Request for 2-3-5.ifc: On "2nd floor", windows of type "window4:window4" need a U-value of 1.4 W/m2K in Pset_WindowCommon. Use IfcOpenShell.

First a look at what the model holds.

```python
import ifcopenshell
import ifcopenshell.util.element

model = ifcopenshell.open("2-3-5.ifc")
print(model.schema)
storey = next(s for s in model.by_type("IfcBuildingStorey") if s.Name == "2nd floor")
windows = [e for e in ifcopenshell.util.element.get_decomposition(storey) if e.is_a("IfcWindow")]
seen = {}
for e in windows:
    element_type = ifcopenshell.util.element.get_type(e)
    key = (element_type.Name if element_type != e and element_type else None, ifcopenshell.util.element.get_pset(e, "Pset_WindowCommon", "ThermalTransmittance"))
    seen[key] = seen.get(key, 0) + 1
for (name, value), count in sorted(seen.items(), key=str):
    print(count, "x", name, "|", value)
```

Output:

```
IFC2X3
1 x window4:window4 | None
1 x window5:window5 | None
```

```python
import ifcopenshell
import ifcopenshell.api.pset
import ifcopenshell.util.element

model = ifcopenshell.open("2-3-5.ifc")

storey = next(s for s in model.by_type("IfcBuildingStorey") if s.Name == "2nd floor")
windows = [e for e in ifcopenshell.util.element.get_decomposition(storey) if e.is_a("IfcWindow")]

count = 0
for e in windows:
    element_type = ifcopenshell.util.element.get_type(e)
    if element_type in (None, e) or element_type.Name != "window4:window4":
        continue
    # add_pset returns the element's existing set when there is one.
    pset = ifcopenshell.api.pset.add_pset(model, product=e, name="Pset_WindowCommon")
    ifcopenshell.api.pset.edit_pset(model, pset=pset, properties={"ThermalTransmittance": 1.4})
    count += 1

print(count, "windows updated")

model.write("2-3-5_v2.ifc")
```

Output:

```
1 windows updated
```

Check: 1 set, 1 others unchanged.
